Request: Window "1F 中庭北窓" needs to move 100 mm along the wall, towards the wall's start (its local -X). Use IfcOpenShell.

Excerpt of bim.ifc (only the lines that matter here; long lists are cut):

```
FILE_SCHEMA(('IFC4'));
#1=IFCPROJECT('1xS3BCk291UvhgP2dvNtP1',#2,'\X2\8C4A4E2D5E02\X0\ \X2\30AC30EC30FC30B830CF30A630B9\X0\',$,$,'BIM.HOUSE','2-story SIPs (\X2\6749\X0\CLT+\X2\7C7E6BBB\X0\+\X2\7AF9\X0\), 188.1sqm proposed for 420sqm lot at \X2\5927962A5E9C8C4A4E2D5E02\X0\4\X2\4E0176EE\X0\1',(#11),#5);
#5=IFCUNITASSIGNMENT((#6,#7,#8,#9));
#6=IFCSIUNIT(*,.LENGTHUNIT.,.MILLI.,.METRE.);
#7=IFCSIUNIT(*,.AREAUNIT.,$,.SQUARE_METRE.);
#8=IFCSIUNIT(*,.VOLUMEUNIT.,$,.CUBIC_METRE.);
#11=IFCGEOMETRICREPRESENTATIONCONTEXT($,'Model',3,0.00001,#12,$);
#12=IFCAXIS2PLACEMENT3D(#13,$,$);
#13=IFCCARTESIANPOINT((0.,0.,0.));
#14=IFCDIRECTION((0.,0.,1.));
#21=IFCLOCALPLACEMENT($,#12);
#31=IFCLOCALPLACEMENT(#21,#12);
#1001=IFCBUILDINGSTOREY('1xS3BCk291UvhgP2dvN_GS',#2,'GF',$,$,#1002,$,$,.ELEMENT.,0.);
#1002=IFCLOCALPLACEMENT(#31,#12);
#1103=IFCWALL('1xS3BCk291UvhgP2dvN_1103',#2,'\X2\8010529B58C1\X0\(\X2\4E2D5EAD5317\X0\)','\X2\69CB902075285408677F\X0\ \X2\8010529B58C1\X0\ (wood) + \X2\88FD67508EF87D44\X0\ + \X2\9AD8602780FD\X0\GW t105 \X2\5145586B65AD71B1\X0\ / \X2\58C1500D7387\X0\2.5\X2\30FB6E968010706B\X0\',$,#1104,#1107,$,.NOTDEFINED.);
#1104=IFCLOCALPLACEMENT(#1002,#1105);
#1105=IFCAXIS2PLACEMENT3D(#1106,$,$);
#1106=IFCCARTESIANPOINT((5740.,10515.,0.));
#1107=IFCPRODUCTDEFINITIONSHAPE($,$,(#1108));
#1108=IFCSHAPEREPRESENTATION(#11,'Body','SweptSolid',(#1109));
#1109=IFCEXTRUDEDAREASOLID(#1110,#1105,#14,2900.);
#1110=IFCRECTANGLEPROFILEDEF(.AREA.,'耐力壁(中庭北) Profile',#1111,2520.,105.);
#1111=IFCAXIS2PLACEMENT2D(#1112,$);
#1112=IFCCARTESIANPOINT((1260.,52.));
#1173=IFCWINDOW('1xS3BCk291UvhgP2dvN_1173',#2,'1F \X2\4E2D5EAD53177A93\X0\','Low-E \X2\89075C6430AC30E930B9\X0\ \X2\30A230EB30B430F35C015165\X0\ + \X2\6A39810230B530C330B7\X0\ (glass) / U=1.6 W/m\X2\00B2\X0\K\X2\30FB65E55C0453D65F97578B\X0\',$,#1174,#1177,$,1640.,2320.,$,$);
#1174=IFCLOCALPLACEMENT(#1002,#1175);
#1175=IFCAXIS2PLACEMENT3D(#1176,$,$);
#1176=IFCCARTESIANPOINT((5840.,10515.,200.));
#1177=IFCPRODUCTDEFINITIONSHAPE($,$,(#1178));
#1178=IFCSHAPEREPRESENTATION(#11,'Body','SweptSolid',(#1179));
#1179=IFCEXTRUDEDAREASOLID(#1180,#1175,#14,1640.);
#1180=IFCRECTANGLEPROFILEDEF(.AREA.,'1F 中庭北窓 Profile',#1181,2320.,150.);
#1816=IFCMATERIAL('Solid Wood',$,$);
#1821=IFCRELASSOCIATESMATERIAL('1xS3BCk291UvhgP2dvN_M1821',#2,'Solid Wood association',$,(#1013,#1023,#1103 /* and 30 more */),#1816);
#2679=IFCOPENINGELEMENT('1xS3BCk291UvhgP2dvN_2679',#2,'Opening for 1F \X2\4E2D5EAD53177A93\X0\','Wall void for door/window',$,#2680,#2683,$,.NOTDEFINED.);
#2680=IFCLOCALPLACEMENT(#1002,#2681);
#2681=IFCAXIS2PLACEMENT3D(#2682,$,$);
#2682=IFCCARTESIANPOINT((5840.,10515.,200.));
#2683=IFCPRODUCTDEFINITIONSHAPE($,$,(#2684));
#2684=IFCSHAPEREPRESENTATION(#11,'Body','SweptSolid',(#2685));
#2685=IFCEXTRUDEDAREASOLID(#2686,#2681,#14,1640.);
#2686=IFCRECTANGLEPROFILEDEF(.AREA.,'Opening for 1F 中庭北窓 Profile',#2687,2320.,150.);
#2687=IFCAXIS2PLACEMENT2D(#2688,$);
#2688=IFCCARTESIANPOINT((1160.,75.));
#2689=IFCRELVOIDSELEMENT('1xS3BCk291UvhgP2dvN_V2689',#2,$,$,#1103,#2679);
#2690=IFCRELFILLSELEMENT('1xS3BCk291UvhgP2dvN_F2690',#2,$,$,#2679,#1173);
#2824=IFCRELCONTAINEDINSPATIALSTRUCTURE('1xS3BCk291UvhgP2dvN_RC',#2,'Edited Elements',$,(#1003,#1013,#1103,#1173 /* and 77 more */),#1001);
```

```python
import ifcopenshell
import ifcopenshell.api.geometry
import ifcopenshell.util.placement
import ifcopenshell.util.unit

model = ifcopenshell.open("bim.ifc")
unit_scale = ifcopenshell.util.unit.calculate_unit_scale(model)

window = model.by_guid("1xS3BCk291UvhgP2dvN_1173")
opening = window.FillsVoids[0].RelatingOpeningElement
wall = opening.VoidsElements[0].RelatingBuildingElement

wall_matrix = ifcopenshell.util.placement.get_local_placement(wall.ObjectPlacement)
shift = wall_matrix[:3, 0] * -0.1 / unit_scale
before = ifcopenshell.util.placement.get_local_placement(window.ObjectPlacement)[:3, 3].copy()

# The window is not placed relative to its opening, so move both.
for product in (opening, window):
    matrix = ifcopenshell.util.placement.get_local_placement(product.ObjectPlacement)
    matrix[:3, 3] += shift
    ifcopenshell.api.geometry.edit_object_placement(model, product=product, matrix=matrix, is_si=False)

after = ifcopenshell.util.placement.get_local_placement(window.ObjectPlacement)[:3, 3]
print("window moved by", (after - before).round(3) + 0.0)

model.write("bim_rev.ifc")
```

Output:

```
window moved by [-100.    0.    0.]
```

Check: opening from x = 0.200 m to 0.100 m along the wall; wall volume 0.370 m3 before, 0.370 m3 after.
